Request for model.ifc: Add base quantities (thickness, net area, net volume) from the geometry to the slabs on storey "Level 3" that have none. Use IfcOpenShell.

First a look at what the model holds.

```python
import ifcopenshell
import ifcopenshell.util.element
import ifcopenshell.util.unit

model = ifcopenshell.open("model.ifc")
print(model.schema)
for unit_type in ("LENGTHUNIT", "AREAUNIT", "VOLUMEUNIT"):
    print(unit_type, ifcopenshell.util.unit.calculate_unit_scale(model, unit_type))
storey = next(s for s in model.by_type("IfcBuildingStorey") if s.Name == "Level 3")
slabs = [e for e in ifcopenshell.util.element.get_decomposition(storey) if e.is_a("IfcSlab")]
for e in sorted(slabs, key=lambda e: e.id()):
    print(e.id(), e.is_a(), e.Name, list(ifcopenshell.util.element.get_psets(e, qtos_only=True)), sep=" | ")
```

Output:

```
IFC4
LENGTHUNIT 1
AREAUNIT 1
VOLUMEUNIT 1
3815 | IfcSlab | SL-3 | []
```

```python
import ifcopenshell
import ifcopenshell.api.pset
import ifcopenshell.geom
import ifcopenshell.util.element
import ifcopenshell.util.shape
import ifcopenshell.util.unit

model = ifcopenshell.open("model.ifc")
unit_scale = ifcopenshell.util.unit.calculate_unit_scale(model)
area_scale = ifcopenshell.util.unit.calculate_unit_scale(model, "AREAUNIT")
volume_scale = ifcopenshell.util.unit.calculate_unit_scale(model, "VOLUMEUNIT")
settings = ifcopenshell.geom.settings()

storey = next(s for s in model.by_type("IfcBuildingStorey") if s.Name == "Level 3")
slabs = [e for e in ifcopenshell.util.element.get_decomposition(storey) if e.is_a("IfcSlab")]

for e in sorted(slabs, key=lambda e: e.id()):
    if ifcopenshell.util.element.get_psets(e, qtos_only=True, should_inherit=False):
        continue
    # Geometry comes back in metres, in the element's own axes.
    shape = ifcopenshell.geom.create_shape(settings, e)
    values = {
        "Width": ifcopenshell.util.shape.get_z(shape.geometry) / unit_scale,
        "NetArea": ifcopenshell.util.shape.get_footprint_area(shape.geometry) / area_scale,
        "NetVolume": ifcopenshell.util.shape.get_volume(shape.geometry) / volume_scale,
    }
    qto = ifcopenshell.api.pset.add_qto(model, product=e, name="Qto_SlabBaseQuantities")
    ifcopenshell.api.pset.edit_qto(model, qto=qto, properties=values)
    print(e.id(), {k: round(v, 3) for k, v in values.items()})

model.write("model_edited.ifc")
```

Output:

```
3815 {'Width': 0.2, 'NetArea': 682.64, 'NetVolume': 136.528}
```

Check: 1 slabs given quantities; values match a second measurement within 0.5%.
